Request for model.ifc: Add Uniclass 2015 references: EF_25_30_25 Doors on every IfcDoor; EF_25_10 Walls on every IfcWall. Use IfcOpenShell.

First a look at what the model holds.

```python
import ifcopenshell

model = ifcopenshell.open("model.ifc")
print(model.schema)
print("classifications:", [c.Name for c in model.by_type("IfcClassification")])
for ifc_class in ("IfcDoor", "IfcRoof", "IfcStair", "IfcWall", "IfcWindow"):
    print(ifc_class, len(model.by_type(ifc_class)))
```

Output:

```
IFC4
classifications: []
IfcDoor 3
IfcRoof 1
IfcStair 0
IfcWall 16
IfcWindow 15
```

```python
import ifcopenshell
import ifcopenshell.api.classification

model = ifcopenshell.open("model.ifc")

system = ifcopenshell.api.classification.add_classification(model, classification="Uniclass 2015")

codes = {
    "IfcDoor": ("EF_25_30_25", "Doors"),
    "IfcWall": ("EF_25_10", "Walls"),
}
for ifc_class, (code, name) in codes.items():
    products = model.by_type(ifc_class)
    ifcopenshell.api.classification.add_reference(
        model, products=products, classification=system, identification=code, name=name
    )
    print(code, len(products))

model.write("model-out.ifc")
```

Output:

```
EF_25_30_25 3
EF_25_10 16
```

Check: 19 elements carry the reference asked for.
